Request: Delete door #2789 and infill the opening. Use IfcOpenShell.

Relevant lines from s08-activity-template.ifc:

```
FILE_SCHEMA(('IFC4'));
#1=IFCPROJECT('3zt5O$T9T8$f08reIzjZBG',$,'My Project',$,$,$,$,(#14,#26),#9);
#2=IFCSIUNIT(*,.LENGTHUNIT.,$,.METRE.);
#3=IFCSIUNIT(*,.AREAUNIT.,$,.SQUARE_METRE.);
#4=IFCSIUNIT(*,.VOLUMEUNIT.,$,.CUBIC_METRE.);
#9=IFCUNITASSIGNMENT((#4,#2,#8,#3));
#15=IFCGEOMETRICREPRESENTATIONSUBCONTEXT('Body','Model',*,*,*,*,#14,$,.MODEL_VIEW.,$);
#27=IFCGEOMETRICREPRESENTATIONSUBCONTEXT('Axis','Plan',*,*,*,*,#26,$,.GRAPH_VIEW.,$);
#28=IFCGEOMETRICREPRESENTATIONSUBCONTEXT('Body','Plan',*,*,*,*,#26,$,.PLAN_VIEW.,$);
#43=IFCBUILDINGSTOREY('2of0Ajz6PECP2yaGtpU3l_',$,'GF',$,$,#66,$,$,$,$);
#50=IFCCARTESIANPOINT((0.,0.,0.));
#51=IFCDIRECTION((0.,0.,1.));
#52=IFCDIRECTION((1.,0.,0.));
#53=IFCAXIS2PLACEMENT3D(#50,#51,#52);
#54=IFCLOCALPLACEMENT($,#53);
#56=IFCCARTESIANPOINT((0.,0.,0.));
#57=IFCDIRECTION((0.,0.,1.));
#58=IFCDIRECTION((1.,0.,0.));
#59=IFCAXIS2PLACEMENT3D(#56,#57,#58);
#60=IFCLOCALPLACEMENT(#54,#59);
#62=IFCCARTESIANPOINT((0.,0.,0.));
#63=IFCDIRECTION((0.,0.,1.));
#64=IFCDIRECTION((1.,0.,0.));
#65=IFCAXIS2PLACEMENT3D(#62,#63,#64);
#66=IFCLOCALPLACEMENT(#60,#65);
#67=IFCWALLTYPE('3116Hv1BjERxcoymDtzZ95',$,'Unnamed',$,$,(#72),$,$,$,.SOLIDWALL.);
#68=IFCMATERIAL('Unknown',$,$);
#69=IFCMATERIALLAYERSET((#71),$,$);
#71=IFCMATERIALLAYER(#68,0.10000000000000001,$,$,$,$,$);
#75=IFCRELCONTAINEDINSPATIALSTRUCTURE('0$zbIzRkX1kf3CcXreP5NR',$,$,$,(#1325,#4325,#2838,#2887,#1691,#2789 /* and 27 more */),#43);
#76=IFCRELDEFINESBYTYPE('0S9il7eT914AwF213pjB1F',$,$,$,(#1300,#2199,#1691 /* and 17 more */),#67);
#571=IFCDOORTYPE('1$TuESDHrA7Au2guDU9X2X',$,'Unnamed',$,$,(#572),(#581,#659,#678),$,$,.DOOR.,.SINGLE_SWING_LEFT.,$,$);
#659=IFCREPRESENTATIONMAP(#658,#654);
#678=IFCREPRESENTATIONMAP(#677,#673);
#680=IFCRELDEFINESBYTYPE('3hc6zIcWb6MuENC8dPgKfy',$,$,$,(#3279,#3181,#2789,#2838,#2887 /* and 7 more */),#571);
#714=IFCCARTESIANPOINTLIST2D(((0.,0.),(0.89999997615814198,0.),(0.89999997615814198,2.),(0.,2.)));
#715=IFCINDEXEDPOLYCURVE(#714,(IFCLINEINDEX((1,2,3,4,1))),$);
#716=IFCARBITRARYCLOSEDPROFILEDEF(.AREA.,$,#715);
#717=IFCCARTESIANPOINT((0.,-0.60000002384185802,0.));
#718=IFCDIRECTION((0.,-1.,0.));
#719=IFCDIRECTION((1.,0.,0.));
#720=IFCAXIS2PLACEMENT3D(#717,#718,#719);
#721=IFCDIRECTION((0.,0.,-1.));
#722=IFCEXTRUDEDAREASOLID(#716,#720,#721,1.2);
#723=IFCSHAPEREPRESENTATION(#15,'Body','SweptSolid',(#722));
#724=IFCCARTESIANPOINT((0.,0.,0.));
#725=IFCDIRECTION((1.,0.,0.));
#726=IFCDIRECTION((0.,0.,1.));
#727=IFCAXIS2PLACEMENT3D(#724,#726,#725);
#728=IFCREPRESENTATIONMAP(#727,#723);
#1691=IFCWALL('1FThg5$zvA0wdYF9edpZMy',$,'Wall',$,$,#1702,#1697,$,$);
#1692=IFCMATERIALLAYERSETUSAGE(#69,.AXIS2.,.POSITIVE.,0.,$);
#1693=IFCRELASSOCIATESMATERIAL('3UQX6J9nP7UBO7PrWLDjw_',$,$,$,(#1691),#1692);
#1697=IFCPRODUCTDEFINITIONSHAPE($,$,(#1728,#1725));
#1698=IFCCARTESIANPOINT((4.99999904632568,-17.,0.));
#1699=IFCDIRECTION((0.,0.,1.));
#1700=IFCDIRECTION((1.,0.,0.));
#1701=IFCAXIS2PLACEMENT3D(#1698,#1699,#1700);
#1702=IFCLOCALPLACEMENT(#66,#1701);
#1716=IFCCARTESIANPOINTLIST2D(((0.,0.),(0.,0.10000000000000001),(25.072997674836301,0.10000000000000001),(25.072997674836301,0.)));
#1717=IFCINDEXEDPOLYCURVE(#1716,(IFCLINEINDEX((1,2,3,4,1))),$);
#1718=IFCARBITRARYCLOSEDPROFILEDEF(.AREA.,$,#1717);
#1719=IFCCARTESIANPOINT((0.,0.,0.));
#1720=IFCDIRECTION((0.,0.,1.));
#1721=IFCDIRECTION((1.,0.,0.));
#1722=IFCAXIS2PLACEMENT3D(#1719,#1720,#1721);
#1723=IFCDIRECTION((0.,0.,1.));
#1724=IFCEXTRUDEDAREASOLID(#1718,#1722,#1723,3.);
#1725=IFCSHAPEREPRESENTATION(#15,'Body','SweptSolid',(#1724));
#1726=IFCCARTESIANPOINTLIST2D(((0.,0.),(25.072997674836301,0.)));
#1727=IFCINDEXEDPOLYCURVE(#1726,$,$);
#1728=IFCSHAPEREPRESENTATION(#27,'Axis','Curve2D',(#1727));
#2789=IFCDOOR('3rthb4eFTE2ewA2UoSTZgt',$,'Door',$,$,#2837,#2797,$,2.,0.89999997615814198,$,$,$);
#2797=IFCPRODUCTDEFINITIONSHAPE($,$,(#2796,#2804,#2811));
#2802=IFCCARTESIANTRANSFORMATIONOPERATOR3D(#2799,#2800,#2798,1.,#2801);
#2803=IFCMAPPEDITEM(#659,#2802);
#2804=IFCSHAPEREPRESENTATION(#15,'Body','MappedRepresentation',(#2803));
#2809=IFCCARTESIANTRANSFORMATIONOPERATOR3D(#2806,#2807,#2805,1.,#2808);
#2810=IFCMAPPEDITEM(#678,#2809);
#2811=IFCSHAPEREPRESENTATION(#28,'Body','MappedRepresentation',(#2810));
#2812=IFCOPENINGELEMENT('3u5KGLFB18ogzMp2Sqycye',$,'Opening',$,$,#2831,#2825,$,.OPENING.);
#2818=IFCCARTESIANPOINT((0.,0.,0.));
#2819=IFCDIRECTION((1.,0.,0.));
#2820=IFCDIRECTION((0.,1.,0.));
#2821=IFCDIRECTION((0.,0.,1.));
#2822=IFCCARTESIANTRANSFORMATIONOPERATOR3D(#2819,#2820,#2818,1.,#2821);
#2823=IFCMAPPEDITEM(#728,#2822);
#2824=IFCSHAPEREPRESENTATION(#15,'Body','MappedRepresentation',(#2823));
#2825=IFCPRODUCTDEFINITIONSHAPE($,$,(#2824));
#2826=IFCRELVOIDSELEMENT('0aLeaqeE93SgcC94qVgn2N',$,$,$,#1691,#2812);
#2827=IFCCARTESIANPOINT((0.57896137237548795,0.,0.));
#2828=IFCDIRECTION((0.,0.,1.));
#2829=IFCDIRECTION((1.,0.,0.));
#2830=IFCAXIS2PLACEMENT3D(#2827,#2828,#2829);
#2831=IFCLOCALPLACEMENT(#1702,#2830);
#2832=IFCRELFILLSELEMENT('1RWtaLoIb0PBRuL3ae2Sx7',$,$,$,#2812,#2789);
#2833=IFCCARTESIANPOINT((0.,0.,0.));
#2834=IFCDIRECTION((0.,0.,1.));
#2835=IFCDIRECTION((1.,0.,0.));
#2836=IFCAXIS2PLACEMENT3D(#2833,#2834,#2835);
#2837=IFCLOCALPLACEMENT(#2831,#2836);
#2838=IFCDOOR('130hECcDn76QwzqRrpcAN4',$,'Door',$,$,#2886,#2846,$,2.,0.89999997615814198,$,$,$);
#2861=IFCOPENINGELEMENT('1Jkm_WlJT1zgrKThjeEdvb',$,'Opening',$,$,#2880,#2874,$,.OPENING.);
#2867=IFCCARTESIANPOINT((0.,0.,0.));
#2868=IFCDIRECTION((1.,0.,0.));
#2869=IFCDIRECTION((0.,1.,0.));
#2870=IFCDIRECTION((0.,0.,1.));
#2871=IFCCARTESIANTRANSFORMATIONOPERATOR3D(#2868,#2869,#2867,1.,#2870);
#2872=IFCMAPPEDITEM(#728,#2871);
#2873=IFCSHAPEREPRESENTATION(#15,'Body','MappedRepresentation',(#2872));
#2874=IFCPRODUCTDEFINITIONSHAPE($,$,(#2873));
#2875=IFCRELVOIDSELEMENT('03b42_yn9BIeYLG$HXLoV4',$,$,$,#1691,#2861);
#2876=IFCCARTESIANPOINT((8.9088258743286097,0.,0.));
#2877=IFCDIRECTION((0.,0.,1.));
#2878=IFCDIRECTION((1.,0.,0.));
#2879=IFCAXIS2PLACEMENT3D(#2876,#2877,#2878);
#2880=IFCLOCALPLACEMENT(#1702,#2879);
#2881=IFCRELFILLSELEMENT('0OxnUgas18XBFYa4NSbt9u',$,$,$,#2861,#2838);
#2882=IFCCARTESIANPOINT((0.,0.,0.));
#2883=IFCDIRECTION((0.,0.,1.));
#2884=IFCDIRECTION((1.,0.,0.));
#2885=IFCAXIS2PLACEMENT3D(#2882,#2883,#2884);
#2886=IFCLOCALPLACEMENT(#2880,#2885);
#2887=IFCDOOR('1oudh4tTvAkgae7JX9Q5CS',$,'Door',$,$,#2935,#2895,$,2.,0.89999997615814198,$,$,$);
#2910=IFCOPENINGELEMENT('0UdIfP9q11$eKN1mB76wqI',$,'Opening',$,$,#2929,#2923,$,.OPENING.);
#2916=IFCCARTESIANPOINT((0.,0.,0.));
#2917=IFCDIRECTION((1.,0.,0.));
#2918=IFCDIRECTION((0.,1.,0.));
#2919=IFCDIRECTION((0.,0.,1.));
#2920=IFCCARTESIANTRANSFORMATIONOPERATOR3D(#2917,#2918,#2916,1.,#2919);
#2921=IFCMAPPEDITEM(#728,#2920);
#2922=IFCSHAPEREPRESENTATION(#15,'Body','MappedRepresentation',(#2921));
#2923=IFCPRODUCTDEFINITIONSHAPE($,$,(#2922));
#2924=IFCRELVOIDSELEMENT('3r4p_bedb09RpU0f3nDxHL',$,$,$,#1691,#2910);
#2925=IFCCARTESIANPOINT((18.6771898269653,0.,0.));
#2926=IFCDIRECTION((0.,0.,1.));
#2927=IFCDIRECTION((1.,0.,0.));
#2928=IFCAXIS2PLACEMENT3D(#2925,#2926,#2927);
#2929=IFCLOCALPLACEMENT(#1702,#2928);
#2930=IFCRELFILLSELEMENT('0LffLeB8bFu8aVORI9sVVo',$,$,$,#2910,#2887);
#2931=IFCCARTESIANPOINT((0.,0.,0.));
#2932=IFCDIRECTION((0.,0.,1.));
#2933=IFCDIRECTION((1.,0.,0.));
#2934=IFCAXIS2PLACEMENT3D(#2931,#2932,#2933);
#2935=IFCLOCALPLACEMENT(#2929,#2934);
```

```python
import ifcopenshell
import ifcopenshell.api.feature
import ifcopenshell.api.root
import ifcopenshell.geom
import ifcopenshell.util.shape

model = ifcopenshell.open("s08-activity-template.ifc")
settings = ifcopenshell.geom.settings()


def volume(element):
    """Net volume in cubic metres, openings subtracted."""
    shape = ifcopenshell.geom.create_shape(settings, element)
    return ifcopenshell.util.shape.get_volume(shape.geometry)


door = model.by_guid("3rthb4eFTE2ewA2UoSTZgt")
opening = door.FillsVoids[0].RelatingOpeningElement
wall = opening.VoidsElements[0].RelatingBuildingElement
before = volume(wall)

ifcopenshell.api.root.remove_product(model, product=door)
ifcopenshell.api.feature.remove_feature(model, feature=opening)

after = volume(wall)

print(f"wall volume {before:.3f} -> {after:.3f} m3")

model.write("s08-activity-template_edited.ifc")
```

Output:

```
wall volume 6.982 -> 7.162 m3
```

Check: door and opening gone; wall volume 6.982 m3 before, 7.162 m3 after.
